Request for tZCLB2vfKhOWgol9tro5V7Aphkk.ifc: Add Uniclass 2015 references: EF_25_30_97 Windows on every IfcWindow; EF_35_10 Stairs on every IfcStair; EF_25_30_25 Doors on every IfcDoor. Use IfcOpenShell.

First a look at what the model holds.

```python
import ifcopenshell

model = ifcopenshell.open("tZCLB2vfKhOWgol9tro5V7Aphkk.ifc")
print(model.schema)
print("classifications:", [c.Name for c in model.by_type("IfcClassification")])
for ifc_class in ("IfcDoor", "IfcRoof", "IfcStair", "IfcWall", "IfcWindow"):
    print(ifc_class, len(model.by_type(ifc_class)))
```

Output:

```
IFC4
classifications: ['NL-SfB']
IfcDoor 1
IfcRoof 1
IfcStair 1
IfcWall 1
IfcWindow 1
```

```python
import ifcopenshell
import ifcopenshell.api.classification

model = ifcopenshell.open("tZCLB2vfKhOWgol9tro5V7Aphkk.ifc")

system = ifcopenshell.api.classification.add_classification(model, classification="Uniclass 2015")

codes = {
    "IfcWindow": ("EF_25_30_97", "Windows"),
    "IfcStair": ("EF_35_10", "Stairs"),
    "IfcDoor": ("EF_25_30_25", "Doors"),
}
for ifc_class, (code, name) in codes.items():
    products = model.by_type(ifc_class)
    ifcopenshell.api.classification.add_reference(
        model, products=products, classification=system, identification=code, name=name
    )
    print(code, len(products))

model.write("tZCLB2vfKhOWgol9tro5V7Aphkk_updated.ifc")
```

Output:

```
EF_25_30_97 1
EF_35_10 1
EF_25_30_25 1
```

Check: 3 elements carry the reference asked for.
